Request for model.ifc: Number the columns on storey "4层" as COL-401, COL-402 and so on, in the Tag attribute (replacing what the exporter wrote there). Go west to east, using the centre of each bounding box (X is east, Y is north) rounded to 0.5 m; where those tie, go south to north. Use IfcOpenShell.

First a look at what the model holds.

```python
import ifcopenshell
import ifcopenshell.util.element
import ifcopenshell.util.placement

model = ifcopenshell.open("model.ifc")
print(model.schema)
storey = next(s for s in model.by_type("IfcBuildingStorey") if s.Name == "4层")
columns = [e for e in ifcopenshell.util.element.get_decomposition(storey) if e.is_a("IfcColumn")]
for e in sorted(columns, key=lambda e: e.id()):
    origin = ifcopenshell.util.placement.get_local_placement(e.ObjectPlacement)[:3, 3]
    print(e.id(), e.Tag, e.Name, origin.round(2) + 0.0, sep=" | ")
```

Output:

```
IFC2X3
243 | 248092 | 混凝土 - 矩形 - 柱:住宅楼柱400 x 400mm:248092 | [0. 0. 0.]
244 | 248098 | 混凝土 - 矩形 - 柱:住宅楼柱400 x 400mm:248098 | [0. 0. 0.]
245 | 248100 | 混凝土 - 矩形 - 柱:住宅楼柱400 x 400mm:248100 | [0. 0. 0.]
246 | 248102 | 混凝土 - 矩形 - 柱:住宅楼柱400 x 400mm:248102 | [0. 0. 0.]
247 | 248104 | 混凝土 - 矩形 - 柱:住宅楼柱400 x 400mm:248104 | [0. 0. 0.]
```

```python
import ifcopenshell
import ifcopenshell.geom
import ifcopenshell.util.element
import ifcopenshell.util.shape

model = ifcopenshell.open("model.ifc")
settings = ifcopenshell.geom.settings()
settings.set("use-world-coords", True)


def centre(element):
    shape = ifcopenshell.geom.create_shape(settings, element)
    return ifcopenshell.util.shape.get_bbox_centroid(shape.geometry)


storey = next(s for s in model.by_type("IfcBuildingStorey") if s.Name == "4层")
columns = [e for e in ifcopenshell.util.element.get_decomposition(storey) if e.is_a("IfcColumn")]

# Insertion points can sit at a corner or the storey origin, so sort by the geometry (in metres).
centres = {e: centre(e) for e in columns}
columns.sort(key=lambda e: (round(centres[e][0] / 0.5), centres[e][1]))

for i, e in enumerate(columns, start=1):
    number = f"COL-4{i:02d}"
    e.Tag = number
    print(e.id(), number)

model.write("model_edited.ifc")
```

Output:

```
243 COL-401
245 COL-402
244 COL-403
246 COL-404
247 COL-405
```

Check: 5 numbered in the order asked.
